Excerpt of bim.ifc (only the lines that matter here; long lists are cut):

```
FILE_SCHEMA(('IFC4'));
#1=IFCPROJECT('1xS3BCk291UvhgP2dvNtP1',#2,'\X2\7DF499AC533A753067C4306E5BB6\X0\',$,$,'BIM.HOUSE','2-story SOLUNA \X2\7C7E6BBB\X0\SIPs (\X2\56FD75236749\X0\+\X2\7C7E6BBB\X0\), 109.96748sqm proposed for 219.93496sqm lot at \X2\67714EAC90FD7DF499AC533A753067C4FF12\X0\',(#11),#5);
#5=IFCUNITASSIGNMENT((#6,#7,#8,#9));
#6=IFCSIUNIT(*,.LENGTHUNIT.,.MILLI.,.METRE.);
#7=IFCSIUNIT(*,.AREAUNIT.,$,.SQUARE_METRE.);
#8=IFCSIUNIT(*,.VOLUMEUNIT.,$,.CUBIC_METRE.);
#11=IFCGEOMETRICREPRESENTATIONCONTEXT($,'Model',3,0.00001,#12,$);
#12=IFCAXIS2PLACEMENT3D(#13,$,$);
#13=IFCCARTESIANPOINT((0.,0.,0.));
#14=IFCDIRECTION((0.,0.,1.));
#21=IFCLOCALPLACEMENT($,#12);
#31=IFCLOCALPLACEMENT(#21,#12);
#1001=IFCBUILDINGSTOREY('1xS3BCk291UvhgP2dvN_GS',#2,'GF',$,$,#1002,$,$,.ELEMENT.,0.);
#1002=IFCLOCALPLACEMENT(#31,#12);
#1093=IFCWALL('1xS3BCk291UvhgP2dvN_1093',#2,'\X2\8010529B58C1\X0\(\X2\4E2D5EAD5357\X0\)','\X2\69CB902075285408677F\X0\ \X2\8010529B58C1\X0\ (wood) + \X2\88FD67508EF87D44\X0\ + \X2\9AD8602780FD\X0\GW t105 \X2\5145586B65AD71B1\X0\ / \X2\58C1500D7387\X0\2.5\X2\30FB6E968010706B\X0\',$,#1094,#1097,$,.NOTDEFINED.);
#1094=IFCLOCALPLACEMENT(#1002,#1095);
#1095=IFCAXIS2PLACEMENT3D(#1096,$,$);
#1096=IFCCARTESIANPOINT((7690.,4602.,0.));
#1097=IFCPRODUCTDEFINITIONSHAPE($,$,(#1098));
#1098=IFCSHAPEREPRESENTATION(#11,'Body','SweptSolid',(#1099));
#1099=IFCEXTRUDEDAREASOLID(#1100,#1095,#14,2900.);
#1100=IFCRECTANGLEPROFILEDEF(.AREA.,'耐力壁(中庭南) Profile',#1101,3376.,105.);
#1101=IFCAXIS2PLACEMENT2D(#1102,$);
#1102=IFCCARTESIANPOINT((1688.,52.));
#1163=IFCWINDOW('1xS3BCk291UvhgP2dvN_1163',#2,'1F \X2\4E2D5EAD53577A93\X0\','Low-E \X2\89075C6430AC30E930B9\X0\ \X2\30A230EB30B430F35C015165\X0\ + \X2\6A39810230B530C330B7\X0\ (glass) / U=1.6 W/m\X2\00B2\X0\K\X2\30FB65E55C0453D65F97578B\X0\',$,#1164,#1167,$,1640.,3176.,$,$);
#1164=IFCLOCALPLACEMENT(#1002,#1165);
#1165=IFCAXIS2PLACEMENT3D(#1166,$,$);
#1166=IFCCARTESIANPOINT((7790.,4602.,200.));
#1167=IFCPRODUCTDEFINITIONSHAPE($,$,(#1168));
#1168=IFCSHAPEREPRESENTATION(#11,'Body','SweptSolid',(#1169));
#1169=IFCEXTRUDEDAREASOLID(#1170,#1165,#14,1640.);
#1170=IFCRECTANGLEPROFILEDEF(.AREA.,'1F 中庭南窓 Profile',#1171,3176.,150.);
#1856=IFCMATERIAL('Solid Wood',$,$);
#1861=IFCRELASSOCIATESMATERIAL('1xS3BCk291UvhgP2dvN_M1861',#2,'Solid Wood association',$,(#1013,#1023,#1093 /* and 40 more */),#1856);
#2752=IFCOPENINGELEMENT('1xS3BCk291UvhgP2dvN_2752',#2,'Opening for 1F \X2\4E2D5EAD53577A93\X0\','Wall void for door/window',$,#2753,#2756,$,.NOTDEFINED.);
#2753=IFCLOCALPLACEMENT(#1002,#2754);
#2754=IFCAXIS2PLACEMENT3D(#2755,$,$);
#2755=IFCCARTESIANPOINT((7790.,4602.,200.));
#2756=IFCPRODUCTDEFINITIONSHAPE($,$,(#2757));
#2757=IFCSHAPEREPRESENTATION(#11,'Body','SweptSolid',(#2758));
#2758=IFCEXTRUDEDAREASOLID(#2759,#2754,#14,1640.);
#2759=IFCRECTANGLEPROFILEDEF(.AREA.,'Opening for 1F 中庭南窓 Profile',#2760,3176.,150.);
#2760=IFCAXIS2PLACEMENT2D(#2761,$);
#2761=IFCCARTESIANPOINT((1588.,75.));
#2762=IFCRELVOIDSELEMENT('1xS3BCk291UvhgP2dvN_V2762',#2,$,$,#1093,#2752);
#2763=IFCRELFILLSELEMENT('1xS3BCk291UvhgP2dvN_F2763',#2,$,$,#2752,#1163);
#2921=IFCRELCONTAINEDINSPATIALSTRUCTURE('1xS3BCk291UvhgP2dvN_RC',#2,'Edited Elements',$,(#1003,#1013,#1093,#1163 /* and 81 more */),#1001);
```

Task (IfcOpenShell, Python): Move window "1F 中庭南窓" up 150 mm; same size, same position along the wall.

```python
import numpy as np
import ifcopenshell
import ifcopenshell.api.geometry
import ifcopenshell.util.placement
import ifcopenshell.util.unit

model = ifcopenshell.open("bim.ifc")
unit_scale = ifcopenshell.util.unit.calculate_unit_scale(model)

window = model.by_id(1163)
opening = window.FillsVoids[0].RelatingOpeningElement
dz = 0.15 / unit_scale

shift = np.array([0.0, 0.0, dz])
# The window is not placed relative to its opening, so move both.
for product in (opening, window):
    matrix = ifcopenshell.util.placement.get_local_placement(product.ObjectPlacement)
    matrix[:3, 3] += shift
    ifcopenshell.api.geometry.edit_object_placement(model, product=product, matrix=matrix, is_si=False)

print(f"moved by {dz * unit_scale:+.3f} m")

model.write("bim_edited.ifc")
```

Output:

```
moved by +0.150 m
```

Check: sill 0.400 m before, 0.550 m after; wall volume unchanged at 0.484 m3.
